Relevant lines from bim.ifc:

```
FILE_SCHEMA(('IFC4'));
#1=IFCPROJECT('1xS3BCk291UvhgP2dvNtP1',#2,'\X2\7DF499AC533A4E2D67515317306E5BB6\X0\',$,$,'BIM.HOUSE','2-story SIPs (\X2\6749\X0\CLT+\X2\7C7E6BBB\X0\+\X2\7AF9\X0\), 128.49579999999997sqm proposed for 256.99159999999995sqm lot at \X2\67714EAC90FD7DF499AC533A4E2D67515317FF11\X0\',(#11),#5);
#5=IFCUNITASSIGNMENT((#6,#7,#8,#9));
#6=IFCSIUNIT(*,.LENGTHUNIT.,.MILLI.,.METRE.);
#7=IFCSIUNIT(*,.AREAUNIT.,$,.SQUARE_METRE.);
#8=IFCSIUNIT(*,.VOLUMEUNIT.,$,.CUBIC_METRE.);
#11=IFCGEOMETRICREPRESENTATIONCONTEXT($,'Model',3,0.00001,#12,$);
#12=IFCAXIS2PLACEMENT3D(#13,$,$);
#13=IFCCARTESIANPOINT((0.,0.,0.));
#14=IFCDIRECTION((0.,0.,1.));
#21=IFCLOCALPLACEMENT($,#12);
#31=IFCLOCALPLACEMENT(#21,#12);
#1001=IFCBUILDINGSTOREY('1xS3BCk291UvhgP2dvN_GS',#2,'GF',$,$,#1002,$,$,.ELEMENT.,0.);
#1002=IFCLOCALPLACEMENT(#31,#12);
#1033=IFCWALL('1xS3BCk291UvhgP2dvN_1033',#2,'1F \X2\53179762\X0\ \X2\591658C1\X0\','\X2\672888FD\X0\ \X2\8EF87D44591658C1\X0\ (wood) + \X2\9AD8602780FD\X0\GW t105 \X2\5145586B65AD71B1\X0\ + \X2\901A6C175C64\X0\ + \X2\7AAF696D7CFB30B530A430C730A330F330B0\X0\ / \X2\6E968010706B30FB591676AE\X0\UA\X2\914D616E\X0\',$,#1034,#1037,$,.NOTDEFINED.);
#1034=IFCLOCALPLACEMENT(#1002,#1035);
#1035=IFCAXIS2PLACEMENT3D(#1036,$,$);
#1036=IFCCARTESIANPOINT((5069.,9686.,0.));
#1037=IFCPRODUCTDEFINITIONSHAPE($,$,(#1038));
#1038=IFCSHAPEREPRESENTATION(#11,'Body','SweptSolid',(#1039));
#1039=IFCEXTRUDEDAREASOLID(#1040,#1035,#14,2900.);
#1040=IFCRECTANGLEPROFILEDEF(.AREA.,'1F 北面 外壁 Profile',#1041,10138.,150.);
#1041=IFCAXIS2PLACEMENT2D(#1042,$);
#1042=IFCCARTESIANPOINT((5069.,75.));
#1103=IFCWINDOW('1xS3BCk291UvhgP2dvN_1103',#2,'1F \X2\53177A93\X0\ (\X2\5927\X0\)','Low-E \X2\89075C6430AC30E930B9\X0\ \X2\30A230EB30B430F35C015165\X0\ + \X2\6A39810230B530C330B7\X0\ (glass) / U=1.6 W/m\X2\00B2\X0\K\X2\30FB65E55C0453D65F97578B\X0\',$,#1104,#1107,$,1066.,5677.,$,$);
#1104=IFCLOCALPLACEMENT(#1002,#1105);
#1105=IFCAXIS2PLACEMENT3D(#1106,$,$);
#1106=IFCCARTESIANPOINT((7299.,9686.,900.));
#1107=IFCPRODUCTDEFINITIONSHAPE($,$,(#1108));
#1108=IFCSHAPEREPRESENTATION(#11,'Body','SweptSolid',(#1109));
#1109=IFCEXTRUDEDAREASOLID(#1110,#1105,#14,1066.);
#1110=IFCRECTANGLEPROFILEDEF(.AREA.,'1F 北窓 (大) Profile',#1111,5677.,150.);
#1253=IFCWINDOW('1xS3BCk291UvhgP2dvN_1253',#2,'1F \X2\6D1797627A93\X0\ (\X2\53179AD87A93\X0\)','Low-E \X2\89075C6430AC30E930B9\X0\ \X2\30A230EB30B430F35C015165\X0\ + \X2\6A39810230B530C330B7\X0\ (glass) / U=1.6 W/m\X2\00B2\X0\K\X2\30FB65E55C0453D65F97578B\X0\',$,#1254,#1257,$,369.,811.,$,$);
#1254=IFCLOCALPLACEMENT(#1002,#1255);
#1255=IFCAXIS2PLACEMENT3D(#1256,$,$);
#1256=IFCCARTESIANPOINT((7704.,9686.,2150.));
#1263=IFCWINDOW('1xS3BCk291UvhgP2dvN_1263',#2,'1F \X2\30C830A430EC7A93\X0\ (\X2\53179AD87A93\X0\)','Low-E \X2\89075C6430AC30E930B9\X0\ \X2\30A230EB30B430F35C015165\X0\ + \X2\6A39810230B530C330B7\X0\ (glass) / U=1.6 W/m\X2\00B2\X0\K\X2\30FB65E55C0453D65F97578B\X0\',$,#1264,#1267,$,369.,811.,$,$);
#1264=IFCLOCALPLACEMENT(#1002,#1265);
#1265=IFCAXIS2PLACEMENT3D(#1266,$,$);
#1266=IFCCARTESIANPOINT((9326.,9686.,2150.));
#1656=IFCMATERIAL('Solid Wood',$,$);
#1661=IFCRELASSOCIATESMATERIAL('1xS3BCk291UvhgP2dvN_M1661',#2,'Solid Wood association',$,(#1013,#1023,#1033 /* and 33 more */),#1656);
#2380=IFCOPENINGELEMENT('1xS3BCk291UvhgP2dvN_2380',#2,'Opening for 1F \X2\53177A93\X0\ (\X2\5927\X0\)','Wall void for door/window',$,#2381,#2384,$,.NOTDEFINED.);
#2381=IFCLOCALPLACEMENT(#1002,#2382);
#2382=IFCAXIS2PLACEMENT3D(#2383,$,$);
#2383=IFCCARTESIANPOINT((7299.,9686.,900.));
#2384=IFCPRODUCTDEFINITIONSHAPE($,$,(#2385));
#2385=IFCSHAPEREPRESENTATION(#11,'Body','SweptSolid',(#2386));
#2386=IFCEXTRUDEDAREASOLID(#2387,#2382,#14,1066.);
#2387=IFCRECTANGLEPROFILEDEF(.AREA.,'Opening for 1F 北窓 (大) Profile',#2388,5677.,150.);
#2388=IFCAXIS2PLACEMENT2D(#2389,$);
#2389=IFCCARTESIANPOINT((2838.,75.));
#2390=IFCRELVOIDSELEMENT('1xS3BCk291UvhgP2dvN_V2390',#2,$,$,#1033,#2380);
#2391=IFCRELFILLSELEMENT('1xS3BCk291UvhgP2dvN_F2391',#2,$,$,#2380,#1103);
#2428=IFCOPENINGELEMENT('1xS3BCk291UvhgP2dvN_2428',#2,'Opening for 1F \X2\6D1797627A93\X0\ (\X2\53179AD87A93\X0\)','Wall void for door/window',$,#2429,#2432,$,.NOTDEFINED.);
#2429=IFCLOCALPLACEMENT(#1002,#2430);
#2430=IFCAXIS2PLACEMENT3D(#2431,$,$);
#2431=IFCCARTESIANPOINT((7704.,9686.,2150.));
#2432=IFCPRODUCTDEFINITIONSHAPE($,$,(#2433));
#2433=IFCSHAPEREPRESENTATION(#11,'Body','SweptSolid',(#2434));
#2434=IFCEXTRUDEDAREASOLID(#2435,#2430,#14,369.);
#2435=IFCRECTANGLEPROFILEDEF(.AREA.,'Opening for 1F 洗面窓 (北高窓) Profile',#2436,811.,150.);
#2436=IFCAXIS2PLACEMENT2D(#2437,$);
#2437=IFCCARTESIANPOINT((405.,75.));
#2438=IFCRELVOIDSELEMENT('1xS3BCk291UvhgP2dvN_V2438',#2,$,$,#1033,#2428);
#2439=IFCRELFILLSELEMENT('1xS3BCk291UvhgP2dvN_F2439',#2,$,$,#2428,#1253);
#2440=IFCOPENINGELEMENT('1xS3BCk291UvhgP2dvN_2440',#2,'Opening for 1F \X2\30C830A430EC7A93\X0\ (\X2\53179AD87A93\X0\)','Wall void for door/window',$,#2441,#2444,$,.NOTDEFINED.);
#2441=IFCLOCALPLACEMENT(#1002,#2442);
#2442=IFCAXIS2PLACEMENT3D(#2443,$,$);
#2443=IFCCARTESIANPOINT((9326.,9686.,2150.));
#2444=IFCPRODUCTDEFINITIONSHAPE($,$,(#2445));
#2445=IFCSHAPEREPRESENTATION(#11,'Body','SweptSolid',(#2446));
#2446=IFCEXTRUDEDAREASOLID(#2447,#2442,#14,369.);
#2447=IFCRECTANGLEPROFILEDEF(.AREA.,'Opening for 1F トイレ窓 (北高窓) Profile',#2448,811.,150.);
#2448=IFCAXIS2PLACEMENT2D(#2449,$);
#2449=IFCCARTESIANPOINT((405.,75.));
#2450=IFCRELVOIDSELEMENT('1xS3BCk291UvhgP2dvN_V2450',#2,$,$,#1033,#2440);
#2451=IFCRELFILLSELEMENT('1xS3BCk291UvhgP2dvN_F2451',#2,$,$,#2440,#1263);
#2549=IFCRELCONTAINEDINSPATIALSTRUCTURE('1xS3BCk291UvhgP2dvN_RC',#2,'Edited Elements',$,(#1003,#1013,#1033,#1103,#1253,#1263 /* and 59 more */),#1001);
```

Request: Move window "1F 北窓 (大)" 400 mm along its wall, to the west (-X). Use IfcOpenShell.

```python
import ifcopenshell
import ifcopenshell.api.geometry
import ifcopenshell.util.placement
import ifcopenshell.util.unit

model = ifcopenshell.open("bim.ifc")
unit_scale = ifcopenshell.util.unit.calculate_unit_scale(model)

window = model.by_id(1103)
opening = window.FillsVoids[0].RelatingOpeningElement
wall = opening.VoidsElements[0].RelatingBuildingElement

wall_matrix = ifcopenshell.util.placement.get_local_placement(wall.ObjectPlacement)
shift = wall_matrix[:3, 0] * -0.4 / unit_scale
before = ifcopenshell.util.placement.get_local_placement(window.ObjectPlacement)[:3, 3].copy()

# The window is not placed relative to its opening, so move both.
for product in (opening, window):
    matrix = ifcopenshell.util.placement.get_local_placement(product.ObjectPlacement)
    matrix[:3, 3] += shift
    ifcopenshell.api.geometry.edit_object_placement(model, product=product, matrix=matrix, is_si=False)

after = ifcopenshell.util.placement.get_local_placement(window.ObjectPlacement)[:3, 3]
print("window moved by", (after - before).round(3) + 0.0)

model.write("bim_updated.ifc")
```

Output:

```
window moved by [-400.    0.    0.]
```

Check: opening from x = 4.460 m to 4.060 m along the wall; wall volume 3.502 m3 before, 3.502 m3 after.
